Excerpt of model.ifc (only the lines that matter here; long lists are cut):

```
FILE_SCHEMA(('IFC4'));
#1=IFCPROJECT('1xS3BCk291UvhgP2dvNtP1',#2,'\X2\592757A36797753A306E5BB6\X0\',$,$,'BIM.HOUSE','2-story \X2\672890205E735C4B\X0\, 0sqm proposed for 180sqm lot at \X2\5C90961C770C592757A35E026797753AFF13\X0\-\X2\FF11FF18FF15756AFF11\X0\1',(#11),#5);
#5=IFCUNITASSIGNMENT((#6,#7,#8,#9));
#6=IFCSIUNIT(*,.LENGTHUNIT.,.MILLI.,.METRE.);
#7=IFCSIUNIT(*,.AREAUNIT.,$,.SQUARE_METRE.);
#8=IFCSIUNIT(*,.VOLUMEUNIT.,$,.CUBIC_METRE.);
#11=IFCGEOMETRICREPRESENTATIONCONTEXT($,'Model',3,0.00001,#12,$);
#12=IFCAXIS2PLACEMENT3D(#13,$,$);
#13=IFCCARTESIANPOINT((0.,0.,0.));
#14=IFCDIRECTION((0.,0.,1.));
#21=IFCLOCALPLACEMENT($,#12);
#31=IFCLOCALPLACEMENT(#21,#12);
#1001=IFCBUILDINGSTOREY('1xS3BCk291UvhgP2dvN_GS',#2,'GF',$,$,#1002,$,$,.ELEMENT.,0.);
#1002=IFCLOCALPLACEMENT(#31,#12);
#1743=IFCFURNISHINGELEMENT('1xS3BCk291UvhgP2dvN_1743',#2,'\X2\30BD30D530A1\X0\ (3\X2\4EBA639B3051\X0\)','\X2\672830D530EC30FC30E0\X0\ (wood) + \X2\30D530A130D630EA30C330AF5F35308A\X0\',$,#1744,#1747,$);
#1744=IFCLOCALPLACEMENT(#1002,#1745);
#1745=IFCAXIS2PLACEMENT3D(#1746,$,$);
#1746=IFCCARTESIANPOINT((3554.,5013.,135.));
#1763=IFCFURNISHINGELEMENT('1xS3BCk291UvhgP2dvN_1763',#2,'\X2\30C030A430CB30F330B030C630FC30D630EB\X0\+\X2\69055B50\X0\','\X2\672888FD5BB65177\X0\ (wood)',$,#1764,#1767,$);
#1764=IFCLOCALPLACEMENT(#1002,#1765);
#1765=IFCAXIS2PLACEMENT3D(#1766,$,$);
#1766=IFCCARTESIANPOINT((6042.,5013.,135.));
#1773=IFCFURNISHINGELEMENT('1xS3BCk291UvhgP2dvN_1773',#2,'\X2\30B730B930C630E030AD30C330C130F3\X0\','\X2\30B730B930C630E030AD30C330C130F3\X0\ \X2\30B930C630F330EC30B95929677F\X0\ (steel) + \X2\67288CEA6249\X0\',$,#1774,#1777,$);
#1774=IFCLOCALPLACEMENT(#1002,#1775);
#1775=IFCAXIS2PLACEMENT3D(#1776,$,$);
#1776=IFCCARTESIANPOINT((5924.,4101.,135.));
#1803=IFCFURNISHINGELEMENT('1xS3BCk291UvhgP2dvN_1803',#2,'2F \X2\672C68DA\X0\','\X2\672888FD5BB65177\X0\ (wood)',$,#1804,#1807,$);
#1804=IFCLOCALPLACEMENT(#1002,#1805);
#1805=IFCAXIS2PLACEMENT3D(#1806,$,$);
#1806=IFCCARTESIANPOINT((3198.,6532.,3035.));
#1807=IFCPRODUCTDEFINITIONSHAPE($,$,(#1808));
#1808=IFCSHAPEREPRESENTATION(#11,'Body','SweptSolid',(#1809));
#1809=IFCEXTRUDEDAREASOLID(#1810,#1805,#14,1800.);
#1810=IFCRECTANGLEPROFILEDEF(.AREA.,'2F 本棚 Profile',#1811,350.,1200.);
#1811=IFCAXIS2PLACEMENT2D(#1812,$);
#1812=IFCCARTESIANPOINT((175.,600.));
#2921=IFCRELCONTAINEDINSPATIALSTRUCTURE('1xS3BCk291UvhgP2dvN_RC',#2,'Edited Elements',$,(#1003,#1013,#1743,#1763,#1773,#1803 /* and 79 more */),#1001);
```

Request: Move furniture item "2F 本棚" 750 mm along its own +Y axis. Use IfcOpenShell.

```python
import ifcopenshell
import ifcopenshell.api.geometry
import ifcopenshell.util.placement

model = ifcopenshell.open("model.ifc")

item = model.by_guid("1xS3BCk291UvhgP2dvN_1803")
matrix = ifcopenshell.util.placement.get_local_placement(item.ObjectPlacement)
matrix[:3, 3] += matrix[:3, 1] * 750.0
ifcopenshell.api.geometry.edit_object_placement(model, product=item, matrix=matrix, is_si=False)

print(ifcopenshell.util.placement.get_local_placement(item.ObjectPlacement).round(3) + 0.0)

model.write("model_updated.ifc")
```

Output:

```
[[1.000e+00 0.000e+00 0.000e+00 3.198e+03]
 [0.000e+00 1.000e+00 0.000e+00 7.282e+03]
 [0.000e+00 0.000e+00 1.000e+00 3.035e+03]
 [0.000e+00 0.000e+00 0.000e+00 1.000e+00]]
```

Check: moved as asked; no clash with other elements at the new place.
